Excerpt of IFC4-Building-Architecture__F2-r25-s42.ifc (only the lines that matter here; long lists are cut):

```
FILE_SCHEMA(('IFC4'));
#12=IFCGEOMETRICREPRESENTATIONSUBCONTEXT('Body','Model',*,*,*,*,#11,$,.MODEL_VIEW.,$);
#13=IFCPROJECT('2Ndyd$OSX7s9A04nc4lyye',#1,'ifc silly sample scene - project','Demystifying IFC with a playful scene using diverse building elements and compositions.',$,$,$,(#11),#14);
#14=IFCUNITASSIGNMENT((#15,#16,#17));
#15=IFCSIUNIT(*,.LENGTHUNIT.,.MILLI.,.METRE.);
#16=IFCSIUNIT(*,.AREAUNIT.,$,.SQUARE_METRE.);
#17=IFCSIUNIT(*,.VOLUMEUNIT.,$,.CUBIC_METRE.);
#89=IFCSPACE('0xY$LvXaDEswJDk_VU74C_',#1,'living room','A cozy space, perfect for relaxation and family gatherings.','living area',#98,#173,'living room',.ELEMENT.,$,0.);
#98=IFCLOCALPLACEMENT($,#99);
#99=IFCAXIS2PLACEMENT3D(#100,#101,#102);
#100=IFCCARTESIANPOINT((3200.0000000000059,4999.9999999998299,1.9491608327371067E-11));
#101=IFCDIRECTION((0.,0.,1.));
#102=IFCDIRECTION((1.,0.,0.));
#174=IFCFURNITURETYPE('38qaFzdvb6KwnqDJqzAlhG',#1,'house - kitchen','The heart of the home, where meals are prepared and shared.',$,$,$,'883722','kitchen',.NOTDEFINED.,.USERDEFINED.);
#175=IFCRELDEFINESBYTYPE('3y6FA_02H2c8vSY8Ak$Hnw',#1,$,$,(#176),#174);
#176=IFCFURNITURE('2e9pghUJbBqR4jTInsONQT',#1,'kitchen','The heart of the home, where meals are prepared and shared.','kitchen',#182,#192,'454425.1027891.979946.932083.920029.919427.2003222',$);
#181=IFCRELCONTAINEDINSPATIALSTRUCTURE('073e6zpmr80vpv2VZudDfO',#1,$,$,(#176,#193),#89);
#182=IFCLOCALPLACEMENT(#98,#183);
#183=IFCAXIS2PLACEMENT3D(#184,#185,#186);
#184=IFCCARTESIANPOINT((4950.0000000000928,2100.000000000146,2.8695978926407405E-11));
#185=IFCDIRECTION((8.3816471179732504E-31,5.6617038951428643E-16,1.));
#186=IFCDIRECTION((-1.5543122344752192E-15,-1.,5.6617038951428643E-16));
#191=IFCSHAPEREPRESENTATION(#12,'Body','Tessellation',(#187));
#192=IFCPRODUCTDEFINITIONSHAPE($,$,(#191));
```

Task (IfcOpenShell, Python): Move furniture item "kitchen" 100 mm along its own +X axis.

```python
import ifcopenshell
import ifcopenshell.api.geometry
import ifcopenshell.util.placement

model = ifcopenshell.open("IFC4-Building-Architecture__F2-r25-s42.ifc")

item = model.by_guid("2e9pghUJbBqR4jTInsONQT")
matrix = ifcopenshell.util.placement.get_local_placement(item.ObjectPlacement)
matrix[:3, 3] += matrix[:3, 0] * 100.0
ifcopenshell.api.geometry.edit_object_placement(model, product=item, matrix=matrix, is_si=False)

print(ifcopenshell.util.placement.get_local_placement(item.ObjectPlacement).round(3) + 0.0)

model.write("IFC4-Building-Architecture__F2-r25-s42_edited.ifc")
```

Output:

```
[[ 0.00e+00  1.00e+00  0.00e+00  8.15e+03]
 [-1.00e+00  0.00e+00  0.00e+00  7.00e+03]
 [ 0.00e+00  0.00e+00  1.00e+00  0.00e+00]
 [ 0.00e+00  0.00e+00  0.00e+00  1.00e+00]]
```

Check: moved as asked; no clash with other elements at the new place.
